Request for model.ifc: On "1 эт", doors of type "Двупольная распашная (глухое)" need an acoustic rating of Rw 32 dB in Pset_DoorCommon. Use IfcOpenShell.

First a look at what the model holds.

```python
import ifcopenshell
import ifcopenshell.util.element

model = ifcopenshell.open("model.ifc")
print(model.schema)
storey = next(s for s in model.by_type("IfcBuildingStorey") if s.Name == "1 эт")
doors = [e for e in ifcopenshell.util.element.get_decomposition(storey) if e.is_a("IfcDoor")]
seen = {}
for e in doors:
    element_type = ifcopenshell.util.element.get_type(e)
    key = (element_type.Name if element_type != e and element_type else None, ifcopenshell.util.element.get_pset(e, "Pset_DoorCommon", "AcousticRating"))
    seen[key] = seen.get(key, 0) + 1
for (name, value), count in sorted(seen.items(), key=str):
    print(count, "x", name, "|", value)
```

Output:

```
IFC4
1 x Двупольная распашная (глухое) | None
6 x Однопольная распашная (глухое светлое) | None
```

```python
import ifcopenshell
import ifcopenshell.api.pset
import ifcopenshell.util.element

model = ifcopenshell.open("model.ifc")

storey = next(s for s in model.by_type("IfcBuildingStorey") if s.Name == "1 эт")
doors = [e for e in ifcopenshell.util.element.get_decomposition(storey) if e.is_a("IfcDoor")]

count = 0
for e in doors:
    element_type = ifcopenshell.util.element.get_type(e)
    if element_type in (None, e) or element_type.Name != "Двупольная распашная (глухое)":
        continue
    # add_pset returns the element's existing set when there is one.
    pset = ifcopenshell.api.pset.add_pset(model, product=e, name="Pset_DoorCommon")
    ifcopenshell.api.pset.edit_pset(model, pset=pset, properties={"AcousticRating": "Rw 32 dB"})
    count += 1

print(count, "doors updated")

model.write("model_v2.ifc")
```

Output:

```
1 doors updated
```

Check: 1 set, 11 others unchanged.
